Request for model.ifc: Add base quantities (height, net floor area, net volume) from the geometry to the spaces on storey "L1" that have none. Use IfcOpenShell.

First a look at what the model holds.

```python
import ifcopenshell
import ifcopenshell.util.element
import ifcopenshell.util.unit

model = ifcopenshell.open("model.ifc")
print(model.schema)
for unit_type in ("LENGTHUNIT", "AREAUNIT", "VOLUMEUNIT"):
    print(unit_type, ifcopenshell.util.unit.calculate_unit_scale(model, unit_type))
storey = next(s for s in model.by_type("IfcBuildingStorey") if s.Name == "L1")
spaces = [e for e in ifcopenshell.util.element.get_decomposition(storey) if e.is_a("IfcSpace")]
for e in sorted(spaces, key=lambda e: e.id()):
    print(e.id(), e.is_a(), e.Name, list(ifcopenshell.util.element.get_psets(e, qtos_only=True)), sep=" | ")
```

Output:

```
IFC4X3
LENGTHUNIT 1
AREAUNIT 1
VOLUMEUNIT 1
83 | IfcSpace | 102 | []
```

```python
import ifcopenshell
import ifcopenshell.api.pset
import ifcopenshell.geom
import ifcopenshell.util.element
import ifcopenshell.util.shape
import ifcopenshell.util.unit

model = ifcopenshell.open("model.ifc")
unit_scale = ifcopenshell.util.unit.calculate_unit_scale(model)
area_scale = ifcopenshell.util.unit.calculate_unit_scale(model, "AREAUNIT")
volume_scale = ifcopenshell.util.unit.calculate_unit_scale(model, "VOLUMEUNIT")
settings = ifcopenshell.geom.settings()

storey = next(s for s in model.by_type("IfcBuildingStorey") if s.Name == "L1")
spaces = [e for e in ifcopenshell.util.element.get_decomposition(storey) if e.is_a("IfcSpace")]

for e in sorted(spaces, key=lambda e: e.id()):
    if ifcopenshell.util.element.get_psets(e, qtos_only=True, should_inherit=False):
        continue
    # Geometry comes back in metres, in the element's own axes.
    shape = ifcopenshell.geom.create_shape(settings, e)
    values = {
        "Height": ifcopenshell.util.shape.get_z(shape.geometry) / unit_scale,
        "NetFloorArea": ifcopenshell.util.shape.get_footprint_area(shape.geometry) / area_scale,
        "NetVolume": ifcopenshell.util.shape.get_volume(shape.geometry) / volume_scale,
    }
    qto = ifcopenshell.api.pset.add_qto(model, product=e, name="Qto_SpaceBaseQuantities")
    ifcopenshell.api.pset.edit_qto(model, qto=qto, properties=values)
    print(e.id(), {k: round(v, 3) for k, v in values.items()})

model.write("model_edited.ifc")
```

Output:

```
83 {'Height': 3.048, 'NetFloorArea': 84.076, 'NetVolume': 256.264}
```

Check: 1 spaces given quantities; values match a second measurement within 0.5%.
